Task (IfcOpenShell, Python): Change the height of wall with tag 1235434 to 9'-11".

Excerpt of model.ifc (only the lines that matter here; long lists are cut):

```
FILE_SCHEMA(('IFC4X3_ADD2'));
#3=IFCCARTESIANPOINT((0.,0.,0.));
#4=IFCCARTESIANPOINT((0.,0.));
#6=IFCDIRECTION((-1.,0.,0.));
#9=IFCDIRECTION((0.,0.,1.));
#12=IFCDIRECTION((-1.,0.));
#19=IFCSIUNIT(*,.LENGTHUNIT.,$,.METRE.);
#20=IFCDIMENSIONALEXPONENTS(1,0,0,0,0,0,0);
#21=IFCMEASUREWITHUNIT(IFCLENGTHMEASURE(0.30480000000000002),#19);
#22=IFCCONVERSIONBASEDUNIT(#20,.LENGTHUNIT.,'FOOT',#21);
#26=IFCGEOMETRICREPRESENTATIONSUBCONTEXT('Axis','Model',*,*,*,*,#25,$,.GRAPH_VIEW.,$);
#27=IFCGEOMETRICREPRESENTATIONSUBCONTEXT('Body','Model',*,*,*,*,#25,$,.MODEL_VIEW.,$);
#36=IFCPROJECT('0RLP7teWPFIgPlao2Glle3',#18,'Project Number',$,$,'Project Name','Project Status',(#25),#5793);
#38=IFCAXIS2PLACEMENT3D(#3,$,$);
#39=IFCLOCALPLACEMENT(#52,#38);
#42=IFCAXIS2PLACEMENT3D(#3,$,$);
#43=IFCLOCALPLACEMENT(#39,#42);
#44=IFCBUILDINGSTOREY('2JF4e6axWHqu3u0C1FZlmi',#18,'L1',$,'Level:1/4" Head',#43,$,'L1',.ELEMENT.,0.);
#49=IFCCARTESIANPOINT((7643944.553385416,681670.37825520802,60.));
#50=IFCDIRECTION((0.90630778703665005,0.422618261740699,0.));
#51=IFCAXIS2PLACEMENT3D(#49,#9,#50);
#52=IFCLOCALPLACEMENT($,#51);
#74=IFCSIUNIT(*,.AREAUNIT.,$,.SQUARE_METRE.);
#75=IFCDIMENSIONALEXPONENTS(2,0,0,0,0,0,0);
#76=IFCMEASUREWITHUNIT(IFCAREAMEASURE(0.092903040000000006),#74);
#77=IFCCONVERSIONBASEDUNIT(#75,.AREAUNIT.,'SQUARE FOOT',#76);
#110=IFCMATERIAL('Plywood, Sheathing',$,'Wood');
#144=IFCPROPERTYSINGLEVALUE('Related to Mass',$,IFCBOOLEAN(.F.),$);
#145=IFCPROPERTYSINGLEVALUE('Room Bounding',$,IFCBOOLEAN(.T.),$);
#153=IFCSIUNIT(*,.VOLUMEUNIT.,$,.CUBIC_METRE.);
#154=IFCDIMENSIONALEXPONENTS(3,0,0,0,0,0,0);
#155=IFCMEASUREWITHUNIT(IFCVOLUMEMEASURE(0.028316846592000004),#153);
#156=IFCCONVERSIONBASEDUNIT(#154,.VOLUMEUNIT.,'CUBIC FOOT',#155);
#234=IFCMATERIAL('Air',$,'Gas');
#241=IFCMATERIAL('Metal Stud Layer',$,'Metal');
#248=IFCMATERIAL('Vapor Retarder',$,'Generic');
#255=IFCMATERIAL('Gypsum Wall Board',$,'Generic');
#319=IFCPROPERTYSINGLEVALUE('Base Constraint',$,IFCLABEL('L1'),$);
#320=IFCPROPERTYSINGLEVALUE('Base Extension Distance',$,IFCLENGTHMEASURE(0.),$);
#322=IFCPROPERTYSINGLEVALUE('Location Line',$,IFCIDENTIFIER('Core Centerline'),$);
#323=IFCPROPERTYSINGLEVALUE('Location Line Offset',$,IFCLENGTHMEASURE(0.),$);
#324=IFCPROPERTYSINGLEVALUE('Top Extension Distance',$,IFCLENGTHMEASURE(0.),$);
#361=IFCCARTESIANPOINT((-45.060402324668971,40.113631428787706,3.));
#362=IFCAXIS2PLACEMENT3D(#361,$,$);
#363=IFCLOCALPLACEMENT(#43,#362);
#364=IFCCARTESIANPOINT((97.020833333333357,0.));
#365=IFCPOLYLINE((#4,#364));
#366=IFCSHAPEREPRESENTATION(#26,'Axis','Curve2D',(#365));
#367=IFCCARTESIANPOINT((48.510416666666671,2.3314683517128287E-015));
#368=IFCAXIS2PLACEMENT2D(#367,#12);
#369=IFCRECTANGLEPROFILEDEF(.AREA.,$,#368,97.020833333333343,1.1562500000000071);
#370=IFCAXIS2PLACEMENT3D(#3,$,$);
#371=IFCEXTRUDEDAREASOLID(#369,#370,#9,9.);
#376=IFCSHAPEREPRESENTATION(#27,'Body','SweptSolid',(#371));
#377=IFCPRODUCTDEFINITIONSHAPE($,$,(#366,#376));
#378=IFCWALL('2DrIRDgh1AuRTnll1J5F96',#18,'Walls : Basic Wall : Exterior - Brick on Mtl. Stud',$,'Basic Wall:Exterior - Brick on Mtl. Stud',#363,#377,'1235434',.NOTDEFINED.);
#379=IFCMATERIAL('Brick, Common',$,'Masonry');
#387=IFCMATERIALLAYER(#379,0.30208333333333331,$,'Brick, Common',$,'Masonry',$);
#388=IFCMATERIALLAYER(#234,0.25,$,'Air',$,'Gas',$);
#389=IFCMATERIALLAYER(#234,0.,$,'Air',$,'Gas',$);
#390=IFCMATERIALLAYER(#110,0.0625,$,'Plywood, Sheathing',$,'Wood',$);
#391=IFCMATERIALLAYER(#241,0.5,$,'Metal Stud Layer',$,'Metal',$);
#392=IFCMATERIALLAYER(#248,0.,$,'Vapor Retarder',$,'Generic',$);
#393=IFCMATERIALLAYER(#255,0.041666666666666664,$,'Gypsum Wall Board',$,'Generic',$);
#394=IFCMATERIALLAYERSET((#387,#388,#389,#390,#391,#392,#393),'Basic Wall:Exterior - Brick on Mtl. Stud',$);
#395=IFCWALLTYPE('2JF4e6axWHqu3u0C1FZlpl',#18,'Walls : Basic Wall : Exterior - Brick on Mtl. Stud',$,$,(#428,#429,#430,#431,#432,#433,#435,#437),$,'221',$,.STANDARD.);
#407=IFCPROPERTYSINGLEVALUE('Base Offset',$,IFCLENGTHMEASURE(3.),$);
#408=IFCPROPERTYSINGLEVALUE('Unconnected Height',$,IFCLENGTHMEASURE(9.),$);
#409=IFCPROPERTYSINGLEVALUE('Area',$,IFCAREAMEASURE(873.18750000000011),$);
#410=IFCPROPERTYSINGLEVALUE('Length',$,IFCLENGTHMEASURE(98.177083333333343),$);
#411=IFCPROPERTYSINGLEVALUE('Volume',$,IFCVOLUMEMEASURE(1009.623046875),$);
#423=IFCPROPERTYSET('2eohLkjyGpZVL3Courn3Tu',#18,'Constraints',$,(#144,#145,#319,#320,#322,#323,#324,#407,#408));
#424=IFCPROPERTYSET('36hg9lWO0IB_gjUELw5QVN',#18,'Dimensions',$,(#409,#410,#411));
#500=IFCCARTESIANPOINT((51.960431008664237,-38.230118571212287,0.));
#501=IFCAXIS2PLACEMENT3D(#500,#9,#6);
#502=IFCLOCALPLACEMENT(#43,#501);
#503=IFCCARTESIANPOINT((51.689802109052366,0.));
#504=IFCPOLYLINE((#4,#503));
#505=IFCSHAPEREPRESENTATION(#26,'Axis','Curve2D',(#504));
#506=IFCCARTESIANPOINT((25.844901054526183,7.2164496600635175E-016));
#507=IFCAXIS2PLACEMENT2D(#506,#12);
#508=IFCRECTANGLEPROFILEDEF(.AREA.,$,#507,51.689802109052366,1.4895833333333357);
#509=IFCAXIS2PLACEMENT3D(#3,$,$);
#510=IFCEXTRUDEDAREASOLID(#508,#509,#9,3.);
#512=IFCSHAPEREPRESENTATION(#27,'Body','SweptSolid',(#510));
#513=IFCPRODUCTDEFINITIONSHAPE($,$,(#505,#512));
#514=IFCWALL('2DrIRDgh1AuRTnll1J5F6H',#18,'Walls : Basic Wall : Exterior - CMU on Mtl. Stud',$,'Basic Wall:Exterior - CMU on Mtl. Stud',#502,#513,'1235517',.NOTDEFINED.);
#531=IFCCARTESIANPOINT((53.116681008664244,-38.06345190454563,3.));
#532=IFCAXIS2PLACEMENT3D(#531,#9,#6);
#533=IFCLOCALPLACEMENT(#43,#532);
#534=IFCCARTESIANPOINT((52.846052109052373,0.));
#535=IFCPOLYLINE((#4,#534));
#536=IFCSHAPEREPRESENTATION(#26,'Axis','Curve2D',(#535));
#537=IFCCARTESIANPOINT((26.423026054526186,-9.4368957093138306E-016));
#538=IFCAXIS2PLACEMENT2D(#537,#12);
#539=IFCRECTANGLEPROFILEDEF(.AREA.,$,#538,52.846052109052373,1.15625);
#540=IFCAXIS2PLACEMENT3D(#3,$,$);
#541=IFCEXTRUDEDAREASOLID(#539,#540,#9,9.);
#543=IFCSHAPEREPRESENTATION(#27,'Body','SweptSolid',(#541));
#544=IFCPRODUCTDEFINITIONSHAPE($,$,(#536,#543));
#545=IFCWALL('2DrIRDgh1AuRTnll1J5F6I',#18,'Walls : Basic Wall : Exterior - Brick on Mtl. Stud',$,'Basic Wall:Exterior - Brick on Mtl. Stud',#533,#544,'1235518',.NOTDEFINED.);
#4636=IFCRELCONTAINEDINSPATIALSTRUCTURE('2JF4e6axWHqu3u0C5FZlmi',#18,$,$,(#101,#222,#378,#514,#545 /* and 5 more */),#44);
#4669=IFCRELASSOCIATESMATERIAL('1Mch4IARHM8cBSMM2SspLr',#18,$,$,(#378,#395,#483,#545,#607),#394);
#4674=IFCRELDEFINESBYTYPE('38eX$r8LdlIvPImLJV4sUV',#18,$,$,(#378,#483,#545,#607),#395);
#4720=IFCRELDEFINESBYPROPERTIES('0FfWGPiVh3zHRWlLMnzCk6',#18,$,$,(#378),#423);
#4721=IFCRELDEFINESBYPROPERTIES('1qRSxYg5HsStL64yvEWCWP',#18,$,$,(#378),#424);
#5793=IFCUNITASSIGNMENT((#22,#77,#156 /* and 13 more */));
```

```python
import ifcopenshell
import ifcopenshell.api.pset
import ifcopenshell.geom
import ifcopenshell.util.element
import ifcopenshell.util.representation
import ifcopenshell.util.shape
import ifcopenshell.util.unit

model = ifcopenshell.open("model.ifc")
unit_scale = ifcopenshell.util.unit.calculate_unit_scale(model)
area_scale = ifcopenshell.util.unit.calculate_unit_scale(model, "AREAUNIT")
volume_scale = ifcopenshell.util.unit.calculate_unit_scale(model, "VOLUMEUNIT")
settings = ifcopenshell.geom.settings()


def volume(element):
    """Net volume in cubic metres, openings subtracted."""
    shape = ifcopenshell.geom.create_shape(settings, element)
    return ifcopenshell.util.shape.get_volume(shape.geometry)


wall = model.by_guid("2DrIRDgh1AuRTnll1J5F96")
before = volume(wall)

body = ifcopenshell.util.representation.get_representation(wall, "Model", "Body")
solid = body.Items[0]
old_height = solid.Depth
solid.Depth = 119 * 0.0254 / unit_scale
after = volume(wall)
thickness = 0.3524  # wall thickness in metres

# Update the stored height, areas and volumes.
pset = model.by_id(ifcopenshell.util.element.get_pset(wall, "Constraints", should_inherit=False)["id"])
ifcopenshell.api.pset.edit_pset(model, pset=pset, properties={
    "Unconnected Height": model.create_entity("IfcLengthMeasure", solid.Depth),
})
pset = model.by_id(ifcopenshell.util.element.get_pset(wall, "Dimensions", should_inherit=False)["id"])
ifcopenshell.api.pset.edit_pset(model, pset=pset, properties={
    "Area": model.create_entity("IfcAreaMeasure", after / thickness / area_scale),
    "Volume": model.create_entity("IfcVolumeMeasure", after / volume_scale),
})

print(f"height {old_height:g} -> {solid.Depth:g}, volume {before:.3f} -> {after:.3f} m3")

model.write("model_rev.ifc")
```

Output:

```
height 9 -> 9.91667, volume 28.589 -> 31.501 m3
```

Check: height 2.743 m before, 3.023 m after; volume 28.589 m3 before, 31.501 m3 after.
